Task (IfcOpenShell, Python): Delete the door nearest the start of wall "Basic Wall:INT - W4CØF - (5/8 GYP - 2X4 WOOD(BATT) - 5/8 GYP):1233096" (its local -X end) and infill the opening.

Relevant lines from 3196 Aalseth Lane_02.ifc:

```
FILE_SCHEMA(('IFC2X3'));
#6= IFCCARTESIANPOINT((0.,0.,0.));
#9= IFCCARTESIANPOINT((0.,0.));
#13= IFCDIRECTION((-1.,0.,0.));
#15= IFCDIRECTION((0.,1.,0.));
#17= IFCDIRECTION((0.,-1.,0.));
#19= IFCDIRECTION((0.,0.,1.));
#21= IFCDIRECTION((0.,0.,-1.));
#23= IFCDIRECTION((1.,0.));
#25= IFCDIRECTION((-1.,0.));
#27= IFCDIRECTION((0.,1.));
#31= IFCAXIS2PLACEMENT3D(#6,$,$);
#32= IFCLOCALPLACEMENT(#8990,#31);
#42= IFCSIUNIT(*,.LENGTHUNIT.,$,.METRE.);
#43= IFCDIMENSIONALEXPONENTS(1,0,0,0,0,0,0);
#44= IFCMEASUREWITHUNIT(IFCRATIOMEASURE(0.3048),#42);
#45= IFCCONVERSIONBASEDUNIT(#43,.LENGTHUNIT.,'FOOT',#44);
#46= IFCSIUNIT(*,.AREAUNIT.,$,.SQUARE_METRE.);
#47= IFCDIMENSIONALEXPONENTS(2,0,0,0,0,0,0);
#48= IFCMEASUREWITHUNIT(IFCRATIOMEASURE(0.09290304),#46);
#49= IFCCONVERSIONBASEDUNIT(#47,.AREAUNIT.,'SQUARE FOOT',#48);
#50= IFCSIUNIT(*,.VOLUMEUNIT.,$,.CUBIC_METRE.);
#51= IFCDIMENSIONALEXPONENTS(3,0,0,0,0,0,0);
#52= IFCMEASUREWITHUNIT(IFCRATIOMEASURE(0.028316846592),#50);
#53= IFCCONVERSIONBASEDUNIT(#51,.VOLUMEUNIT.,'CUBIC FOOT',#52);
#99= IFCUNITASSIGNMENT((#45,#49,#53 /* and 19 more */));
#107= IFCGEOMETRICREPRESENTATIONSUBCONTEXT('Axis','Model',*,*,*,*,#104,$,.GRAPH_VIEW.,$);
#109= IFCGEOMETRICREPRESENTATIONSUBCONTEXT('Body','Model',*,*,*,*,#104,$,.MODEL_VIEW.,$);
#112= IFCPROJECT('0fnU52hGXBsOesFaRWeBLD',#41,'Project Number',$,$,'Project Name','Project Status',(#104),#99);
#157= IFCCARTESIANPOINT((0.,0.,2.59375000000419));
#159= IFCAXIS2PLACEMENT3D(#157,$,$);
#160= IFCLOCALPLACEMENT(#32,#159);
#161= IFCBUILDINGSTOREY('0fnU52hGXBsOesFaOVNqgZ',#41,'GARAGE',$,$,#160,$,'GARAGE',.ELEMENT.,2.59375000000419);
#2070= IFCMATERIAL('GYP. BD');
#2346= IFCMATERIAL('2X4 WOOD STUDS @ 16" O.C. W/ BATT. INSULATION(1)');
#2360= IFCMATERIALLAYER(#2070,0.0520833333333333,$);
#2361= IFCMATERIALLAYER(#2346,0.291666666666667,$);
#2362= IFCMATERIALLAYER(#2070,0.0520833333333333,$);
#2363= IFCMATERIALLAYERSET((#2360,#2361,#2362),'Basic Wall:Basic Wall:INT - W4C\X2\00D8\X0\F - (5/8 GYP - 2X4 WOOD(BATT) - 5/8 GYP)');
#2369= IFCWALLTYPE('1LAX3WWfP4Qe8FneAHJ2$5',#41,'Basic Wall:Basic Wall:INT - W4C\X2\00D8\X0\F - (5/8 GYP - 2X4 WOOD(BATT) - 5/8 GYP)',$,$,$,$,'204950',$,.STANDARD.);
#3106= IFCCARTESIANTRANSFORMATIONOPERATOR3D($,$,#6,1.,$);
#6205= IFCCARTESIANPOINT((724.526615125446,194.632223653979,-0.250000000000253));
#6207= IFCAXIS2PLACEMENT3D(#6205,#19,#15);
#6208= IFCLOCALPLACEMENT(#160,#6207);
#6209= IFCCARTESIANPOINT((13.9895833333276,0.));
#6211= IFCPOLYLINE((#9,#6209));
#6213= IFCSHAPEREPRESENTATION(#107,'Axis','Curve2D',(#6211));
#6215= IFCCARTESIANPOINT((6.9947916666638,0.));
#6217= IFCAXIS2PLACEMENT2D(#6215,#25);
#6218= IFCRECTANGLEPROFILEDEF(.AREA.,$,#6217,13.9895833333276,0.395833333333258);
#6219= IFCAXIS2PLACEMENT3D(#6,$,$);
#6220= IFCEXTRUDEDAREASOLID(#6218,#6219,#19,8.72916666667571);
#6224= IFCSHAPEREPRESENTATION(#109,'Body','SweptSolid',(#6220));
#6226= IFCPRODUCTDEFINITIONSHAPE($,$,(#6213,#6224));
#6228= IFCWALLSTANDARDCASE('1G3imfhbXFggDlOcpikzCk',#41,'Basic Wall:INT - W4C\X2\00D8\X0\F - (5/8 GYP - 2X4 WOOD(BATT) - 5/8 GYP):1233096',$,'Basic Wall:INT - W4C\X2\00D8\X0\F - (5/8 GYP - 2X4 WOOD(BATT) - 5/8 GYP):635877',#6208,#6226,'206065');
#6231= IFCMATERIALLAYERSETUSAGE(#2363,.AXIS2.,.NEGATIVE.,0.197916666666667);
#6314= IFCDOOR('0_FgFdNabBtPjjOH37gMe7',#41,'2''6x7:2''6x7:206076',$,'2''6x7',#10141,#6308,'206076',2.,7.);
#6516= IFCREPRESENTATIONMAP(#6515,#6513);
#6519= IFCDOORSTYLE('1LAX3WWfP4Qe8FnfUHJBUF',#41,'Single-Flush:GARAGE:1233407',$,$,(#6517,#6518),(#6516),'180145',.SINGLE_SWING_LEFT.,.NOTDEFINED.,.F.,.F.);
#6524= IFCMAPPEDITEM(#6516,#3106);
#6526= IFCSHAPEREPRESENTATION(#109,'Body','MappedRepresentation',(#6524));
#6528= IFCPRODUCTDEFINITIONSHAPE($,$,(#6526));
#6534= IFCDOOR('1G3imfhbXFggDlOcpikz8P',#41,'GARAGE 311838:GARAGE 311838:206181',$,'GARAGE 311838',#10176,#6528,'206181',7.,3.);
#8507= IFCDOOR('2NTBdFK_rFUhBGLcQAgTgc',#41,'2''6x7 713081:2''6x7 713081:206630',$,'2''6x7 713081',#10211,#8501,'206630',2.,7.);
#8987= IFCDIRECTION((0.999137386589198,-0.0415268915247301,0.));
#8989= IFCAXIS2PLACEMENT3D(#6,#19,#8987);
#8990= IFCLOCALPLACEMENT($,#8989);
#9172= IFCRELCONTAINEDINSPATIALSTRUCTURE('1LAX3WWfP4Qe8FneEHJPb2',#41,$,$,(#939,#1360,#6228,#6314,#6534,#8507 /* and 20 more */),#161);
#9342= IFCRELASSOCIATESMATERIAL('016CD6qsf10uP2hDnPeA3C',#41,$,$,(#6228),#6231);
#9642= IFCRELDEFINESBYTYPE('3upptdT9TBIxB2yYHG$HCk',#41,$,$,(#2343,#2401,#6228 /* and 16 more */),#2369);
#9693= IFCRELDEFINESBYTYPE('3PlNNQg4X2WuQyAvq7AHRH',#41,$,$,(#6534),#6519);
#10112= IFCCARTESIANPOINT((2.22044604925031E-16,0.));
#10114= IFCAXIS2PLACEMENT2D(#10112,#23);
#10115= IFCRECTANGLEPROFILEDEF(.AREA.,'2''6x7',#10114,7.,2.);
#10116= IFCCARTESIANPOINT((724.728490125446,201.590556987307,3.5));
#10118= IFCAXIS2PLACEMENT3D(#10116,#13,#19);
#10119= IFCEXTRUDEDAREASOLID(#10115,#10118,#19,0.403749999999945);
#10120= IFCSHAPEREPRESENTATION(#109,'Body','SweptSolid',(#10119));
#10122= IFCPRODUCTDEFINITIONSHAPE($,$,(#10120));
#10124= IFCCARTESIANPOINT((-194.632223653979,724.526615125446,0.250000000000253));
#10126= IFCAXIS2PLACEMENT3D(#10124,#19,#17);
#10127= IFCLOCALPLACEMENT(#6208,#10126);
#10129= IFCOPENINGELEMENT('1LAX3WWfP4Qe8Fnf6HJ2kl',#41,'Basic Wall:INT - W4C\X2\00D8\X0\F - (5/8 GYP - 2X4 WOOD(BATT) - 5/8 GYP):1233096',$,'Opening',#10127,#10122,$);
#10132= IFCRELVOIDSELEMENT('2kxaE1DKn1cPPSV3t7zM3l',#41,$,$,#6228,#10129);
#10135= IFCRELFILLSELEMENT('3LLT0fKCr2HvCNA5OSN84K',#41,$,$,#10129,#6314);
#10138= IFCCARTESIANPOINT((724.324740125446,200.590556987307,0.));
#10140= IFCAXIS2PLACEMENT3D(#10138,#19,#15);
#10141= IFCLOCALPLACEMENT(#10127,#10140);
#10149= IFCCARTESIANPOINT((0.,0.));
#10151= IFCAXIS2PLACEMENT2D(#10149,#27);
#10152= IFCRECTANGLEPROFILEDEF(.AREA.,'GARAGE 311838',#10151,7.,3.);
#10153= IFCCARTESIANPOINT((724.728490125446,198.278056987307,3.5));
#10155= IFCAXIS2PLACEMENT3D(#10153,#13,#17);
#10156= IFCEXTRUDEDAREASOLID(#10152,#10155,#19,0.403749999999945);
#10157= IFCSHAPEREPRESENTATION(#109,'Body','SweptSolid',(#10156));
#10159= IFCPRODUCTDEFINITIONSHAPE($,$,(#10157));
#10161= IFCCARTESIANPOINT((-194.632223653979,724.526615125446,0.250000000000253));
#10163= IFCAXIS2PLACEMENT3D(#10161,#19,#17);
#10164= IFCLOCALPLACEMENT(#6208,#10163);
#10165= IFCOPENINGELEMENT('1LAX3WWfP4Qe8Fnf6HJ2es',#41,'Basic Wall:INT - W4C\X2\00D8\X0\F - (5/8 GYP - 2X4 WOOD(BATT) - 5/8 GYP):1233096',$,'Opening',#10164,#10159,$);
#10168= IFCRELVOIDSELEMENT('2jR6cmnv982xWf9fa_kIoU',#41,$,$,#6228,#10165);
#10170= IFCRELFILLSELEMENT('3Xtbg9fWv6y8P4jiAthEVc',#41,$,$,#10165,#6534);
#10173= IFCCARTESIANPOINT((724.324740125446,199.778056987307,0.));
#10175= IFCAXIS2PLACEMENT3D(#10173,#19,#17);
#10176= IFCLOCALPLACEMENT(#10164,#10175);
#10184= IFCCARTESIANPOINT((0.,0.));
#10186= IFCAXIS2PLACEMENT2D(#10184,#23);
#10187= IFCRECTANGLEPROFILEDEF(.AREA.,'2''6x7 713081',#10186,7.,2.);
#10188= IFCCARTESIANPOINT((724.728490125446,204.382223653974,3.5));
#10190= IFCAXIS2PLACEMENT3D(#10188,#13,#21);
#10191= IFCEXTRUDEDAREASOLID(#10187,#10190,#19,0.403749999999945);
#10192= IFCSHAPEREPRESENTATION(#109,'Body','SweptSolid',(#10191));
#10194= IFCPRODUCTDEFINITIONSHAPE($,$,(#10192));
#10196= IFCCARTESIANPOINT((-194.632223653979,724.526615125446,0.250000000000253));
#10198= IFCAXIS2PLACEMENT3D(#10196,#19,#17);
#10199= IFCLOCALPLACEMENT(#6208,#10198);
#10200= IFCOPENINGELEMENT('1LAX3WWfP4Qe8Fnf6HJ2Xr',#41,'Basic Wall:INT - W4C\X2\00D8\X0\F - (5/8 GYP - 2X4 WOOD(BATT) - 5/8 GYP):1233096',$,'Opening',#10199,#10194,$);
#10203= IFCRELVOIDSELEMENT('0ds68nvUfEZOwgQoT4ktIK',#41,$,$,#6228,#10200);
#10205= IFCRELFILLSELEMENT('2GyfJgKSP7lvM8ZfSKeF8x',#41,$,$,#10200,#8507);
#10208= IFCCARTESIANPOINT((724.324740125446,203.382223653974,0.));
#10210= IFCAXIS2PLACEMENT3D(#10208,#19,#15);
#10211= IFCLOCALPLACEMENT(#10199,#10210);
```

```python
import ifcopenshell
import ifcopenshell.api.feature
import ifcopenshell.api.root
import ifcopenshell.geom
import ifcopenshell.util.shape

model = ifcopenshell.open("3196 Aalseth Lane_02.ifc")
settings = ifcopenshell.geom.settings()


def volume(element):
    """Net volume in cubic metres, openings subtracted."""
    shape = ifcopenshell.geom.create_shape(settings, element)
    return ifcopenshell.util.shape.get_volume(shape.geometry)


door = model.by_guid("1G3imfhbXFggDlOcpikz8P")
opening = door.FillsVoids[0].RelatingOpeningElement
wall = opening.VoidsElements[0].RelatingBuildingElement
before = volume(wall)

ifcopenshell.api.root.remove_product(model, product=door)
ifcopenshell.api.feature.remove_feature(model, feature=opening)

after = volume(wall)

print(f"wall volume {before:.3f} -> {after:.3f} m3")

model.write("3196 Aalseth Lane_02_updated.ifc")
```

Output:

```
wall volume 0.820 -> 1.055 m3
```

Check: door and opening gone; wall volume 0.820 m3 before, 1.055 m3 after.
